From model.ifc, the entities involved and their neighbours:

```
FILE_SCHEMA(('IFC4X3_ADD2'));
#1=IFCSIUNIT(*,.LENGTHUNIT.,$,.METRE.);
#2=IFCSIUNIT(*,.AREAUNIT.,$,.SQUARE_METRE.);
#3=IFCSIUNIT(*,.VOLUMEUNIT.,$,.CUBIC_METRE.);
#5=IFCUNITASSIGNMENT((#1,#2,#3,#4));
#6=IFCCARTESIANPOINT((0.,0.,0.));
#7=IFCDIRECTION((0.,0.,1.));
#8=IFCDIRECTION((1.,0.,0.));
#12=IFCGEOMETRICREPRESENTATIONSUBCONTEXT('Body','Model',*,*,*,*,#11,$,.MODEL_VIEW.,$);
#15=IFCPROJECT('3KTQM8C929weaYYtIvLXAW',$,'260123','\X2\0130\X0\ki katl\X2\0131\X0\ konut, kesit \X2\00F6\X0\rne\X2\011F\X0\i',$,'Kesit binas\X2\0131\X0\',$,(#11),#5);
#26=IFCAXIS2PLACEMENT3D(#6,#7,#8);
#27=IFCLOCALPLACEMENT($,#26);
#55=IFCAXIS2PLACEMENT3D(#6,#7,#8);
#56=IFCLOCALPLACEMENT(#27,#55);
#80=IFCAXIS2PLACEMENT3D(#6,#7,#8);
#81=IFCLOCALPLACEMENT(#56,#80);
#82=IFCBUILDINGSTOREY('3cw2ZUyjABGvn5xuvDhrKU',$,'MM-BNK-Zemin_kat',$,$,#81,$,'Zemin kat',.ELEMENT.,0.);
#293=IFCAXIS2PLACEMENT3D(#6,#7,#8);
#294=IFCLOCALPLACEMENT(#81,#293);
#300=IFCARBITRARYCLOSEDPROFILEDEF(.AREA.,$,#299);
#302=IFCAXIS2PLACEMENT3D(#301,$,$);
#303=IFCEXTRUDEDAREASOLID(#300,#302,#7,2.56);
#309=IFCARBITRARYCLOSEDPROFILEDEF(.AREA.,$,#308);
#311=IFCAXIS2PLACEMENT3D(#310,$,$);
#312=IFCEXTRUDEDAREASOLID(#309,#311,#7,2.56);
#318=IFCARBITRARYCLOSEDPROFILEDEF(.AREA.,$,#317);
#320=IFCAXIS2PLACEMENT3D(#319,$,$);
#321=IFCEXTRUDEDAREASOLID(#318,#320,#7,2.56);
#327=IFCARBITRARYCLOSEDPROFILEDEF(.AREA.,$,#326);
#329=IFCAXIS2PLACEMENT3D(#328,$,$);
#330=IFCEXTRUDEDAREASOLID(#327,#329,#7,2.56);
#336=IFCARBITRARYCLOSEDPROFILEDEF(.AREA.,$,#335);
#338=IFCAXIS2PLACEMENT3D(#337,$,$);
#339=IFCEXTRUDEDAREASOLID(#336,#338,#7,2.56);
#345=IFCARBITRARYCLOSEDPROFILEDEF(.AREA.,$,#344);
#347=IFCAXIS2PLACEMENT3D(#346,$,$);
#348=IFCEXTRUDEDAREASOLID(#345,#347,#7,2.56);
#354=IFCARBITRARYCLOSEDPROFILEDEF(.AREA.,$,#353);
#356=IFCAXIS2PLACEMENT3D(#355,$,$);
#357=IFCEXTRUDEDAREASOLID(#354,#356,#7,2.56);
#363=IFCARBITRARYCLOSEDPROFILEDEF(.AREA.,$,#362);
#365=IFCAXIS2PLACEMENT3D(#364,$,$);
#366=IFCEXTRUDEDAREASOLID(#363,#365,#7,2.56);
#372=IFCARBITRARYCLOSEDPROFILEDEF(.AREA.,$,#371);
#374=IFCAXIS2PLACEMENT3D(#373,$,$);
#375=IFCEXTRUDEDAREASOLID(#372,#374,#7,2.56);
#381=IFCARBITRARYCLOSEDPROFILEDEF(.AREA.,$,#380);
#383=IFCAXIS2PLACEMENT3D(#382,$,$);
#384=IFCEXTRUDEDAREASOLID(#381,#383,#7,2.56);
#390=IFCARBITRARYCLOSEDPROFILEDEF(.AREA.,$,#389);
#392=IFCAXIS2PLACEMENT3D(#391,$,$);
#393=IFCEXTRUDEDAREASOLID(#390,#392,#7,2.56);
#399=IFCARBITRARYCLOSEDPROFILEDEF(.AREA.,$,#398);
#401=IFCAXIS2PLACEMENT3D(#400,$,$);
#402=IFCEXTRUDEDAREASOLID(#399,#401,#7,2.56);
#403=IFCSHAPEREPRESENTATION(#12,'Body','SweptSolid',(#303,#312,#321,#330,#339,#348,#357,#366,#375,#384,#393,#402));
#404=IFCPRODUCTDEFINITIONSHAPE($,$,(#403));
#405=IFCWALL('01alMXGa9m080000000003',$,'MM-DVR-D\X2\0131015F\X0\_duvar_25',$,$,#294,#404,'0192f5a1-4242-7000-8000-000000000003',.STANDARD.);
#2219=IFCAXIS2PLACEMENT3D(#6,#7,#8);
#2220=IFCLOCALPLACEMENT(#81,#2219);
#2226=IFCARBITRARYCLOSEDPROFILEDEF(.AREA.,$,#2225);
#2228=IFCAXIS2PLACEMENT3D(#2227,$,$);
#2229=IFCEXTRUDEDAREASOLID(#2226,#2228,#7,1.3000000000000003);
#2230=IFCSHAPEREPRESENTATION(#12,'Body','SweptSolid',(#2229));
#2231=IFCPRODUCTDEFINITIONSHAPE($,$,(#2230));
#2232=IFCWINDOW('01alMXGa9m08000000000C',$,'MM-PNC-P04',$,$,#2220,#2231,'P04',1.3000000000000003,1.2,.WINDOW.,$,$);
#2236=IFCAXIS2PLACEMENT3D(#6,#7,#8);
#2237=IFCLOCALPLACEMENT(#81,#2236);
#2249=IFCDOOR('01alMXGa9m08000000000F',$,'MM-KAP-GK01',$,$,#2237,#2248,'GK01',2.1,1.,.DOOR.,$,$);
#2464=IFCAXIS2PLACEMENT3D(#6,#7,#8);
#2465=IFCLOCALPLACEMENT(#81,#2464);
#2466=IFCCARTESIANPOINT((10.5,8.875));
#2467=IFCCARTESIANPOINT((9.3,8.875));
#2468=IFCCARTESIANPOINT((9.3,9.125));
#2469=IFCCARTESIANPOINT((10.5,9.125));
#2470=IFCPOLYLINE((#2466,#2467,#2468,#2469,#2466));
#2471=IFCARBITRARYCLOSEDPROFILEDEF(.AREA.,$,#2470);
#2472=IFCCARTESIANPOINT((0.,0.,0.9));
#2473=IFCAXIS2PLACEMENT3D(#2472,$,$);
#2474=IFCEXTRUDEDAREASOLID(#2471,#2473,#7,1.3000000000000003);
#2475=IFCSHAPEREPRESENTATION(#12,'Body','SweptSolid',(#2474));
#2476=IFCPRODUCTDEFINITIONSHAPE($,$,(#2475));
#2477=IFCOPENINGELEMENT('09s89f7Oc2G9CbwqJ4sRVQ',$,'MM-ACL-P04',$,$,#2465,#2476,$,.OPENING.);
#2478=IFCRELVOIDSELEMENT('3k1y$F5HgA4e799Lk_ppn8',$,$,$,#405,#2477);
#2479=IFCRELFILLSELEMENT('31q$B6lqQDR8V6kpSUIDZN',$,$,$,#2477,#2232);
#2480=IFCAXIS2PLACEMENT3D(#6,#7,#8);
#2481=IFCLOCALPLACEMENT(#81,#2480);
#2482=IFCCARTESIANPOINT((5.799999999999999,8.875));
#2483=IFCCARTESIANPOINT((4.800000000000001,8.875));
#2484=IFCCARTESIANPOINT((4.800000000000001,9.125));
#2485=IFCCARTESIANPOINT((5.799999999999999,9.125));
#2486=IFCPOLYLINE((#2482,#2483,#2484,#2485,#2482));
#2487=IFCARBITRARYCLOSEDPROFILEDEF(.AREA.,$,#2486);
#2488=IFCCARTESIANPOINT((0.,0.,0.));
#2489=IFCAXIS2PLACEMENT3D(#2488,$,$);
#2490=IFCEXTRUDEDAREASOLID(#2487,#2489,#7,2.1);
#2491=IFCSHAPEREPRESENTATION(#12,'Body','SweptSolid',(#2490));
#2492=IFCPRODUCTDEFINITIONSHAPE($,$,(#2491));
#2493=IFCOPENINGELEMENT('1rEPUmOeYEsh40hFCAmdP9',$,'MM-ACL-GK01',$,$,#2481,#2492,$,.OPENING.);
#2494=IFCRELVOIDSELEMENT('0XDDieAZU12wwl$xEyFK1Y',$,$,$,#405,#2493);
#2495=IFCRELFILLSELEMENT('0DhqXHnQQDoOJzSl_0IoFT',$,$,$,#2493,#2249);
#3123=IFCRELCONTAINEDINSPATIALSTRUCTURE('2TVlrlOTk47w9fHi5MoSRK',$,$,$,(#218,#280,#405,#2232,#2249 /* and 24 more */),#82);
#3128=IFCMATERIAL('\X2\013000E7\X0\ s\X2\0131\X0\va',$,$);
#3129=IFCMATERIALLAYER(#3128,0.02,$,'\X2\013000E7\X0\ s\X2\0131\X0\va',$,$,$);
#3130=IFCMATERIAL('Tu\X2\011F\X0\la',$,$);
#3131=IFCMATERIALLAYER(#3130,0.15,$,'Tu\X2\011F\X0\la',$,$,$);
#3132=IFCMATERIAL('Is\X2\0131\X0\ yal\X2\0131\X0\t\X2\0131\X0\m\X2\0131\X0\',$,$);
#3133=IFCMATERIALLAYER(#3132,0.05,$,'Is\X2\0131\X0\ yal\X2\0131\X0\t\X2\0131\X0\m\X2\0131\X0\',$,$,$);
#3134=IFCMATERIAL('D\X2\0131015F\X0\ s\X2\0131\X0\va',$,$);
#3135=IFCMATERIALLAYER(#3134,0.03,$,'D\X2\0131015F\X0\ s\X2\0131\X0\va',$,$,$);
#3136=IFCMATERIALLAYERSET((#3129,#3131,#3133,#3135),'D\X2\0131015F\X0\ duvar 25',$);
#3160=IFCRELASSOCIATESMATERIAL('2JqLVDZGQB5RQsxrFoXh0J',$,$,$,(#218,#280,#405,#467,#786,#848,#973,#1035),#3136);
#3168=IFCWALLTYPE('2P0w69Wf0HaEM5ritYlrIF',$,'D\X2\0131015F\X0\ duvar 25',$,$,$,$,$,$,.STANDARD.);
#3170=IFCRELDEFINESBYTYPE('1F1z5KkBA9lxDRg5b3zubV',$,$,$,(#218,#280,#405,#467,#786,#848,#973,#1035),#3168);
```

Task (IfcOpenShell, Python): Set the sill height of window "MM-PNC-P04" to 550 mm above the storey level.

```python
import numpy as np
import ifcopenshell
import ifcopenshell.api.geometry
import ifcopenshell.geom
import ifcopenshell.util.element
import ifcopenshell.util.placement
import ifcopenshell.util.shape
import ifcopenshell.util.unit

model = ifcopenshell.open("model.ifc")
unit_scale = ifcopenshell.util.unit.calculate_unit_scale(model)

window = model.by_id(2232)
opening = window.FillsVoids[0].RelatingOpeningElement
storey = ifcopenshell.util.element.get_container(window, ifc_class="IfcBuildingStorey")
level = ifcopenshell.util.placement.get_local_placement(storey.ObjectPlacement)[2, 3]

# The opening's origin need not be at the sill, so measure its lowest point.
shape = ifcopenshell.geom.create_shape(ifcopenshell.geom.settings(), opening)
bottom = ifcopenshell.util.shape.get_shape_bottom_elevation(shape, shape.geometry) / unit_scale
dz = level + 0.55 - bottom

shift = np.array([0.0, 0.0, dz])
# The window is not placed relative to its opening, so move both.
for product in (opening, window):
    matrix = ifcopenshell.util.placement.get_local_placement(product.ObjectPlacement)
    matrix[:3, 3] += shift
    ifcopenshell.api.geometry.edit_object_placement(model, product=product, matrix=matrix, is_si=False)

print(f"moved by {dz * unit_scale:+.3f} m")

model.write("model_v2.ifc")
```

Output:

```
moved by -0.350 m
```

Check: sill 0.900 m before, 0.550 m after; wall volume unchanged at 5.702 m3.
